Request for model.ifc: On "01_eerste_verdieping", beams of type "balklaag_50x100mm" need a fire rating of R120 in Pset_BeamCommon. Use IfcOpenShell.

First a look at what the model holds.

```python
import ifcopenshell
import ifcopenshell.util.element

model = ifcopenshell.open("model.ifc")
print(model.schema)
storey = next(s for s in model.by_type("IfcBuildingStorey") if s.Name == "01_eerste_verdieping")
beams = [e for e in ifcopenshell.util.element.get_decomposition(storey) if e.is_a("IfcBeam")]
seen = {}
for e in beams:
    element_type = ifcopenshell.util.element.get_type(e)
    key = (element_type.Name if element_type != e and element_type else None, ifcopenshell.util.element.get_pset(e, "Pset_BeamCommon", "FireRating"))
    seen[key] = seen.get(key, 0) + 1
for (name, value), count in sorted(seen.items(), key=str):
    print(count, "x", name, "|", value)
```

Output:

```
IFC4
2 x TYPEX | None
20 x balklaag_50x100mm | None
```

```python
import ifcopenshell
import ifcopenshell.api.pset
import ifcopenshell.util.element

model = ifcopenshell.open("model.ifc")

storey = next(s for s in model.by_type("IfcBuildingStorey") if s.Name == "01_eerste_verdieping")
beams = [e for e in ifcopenshell.util.element.get_decomposition(storey) if e.is_a("IfcBeam")]

count = 0
for e in beams:
    element_type = ifcopenshell.util.element.get_type(e)
    if element_type in (None, e) or element_type.Name != "balklaag_50x100mm":
        continue
    # add_pset returns the element's existing set when there is one.
    pset = ifcopenshell.api.pset.add_pset(model, product=e, name="Pset_BeamCommon")
    ifcopenshell.api.pset.edit_pset(model, pset=pset, properties={"FireRating": "R120"})
    count += 1

print(count, "beams updated")

model.write("model-out.ifc")
```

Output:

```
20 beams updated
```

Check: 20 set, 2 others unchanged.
